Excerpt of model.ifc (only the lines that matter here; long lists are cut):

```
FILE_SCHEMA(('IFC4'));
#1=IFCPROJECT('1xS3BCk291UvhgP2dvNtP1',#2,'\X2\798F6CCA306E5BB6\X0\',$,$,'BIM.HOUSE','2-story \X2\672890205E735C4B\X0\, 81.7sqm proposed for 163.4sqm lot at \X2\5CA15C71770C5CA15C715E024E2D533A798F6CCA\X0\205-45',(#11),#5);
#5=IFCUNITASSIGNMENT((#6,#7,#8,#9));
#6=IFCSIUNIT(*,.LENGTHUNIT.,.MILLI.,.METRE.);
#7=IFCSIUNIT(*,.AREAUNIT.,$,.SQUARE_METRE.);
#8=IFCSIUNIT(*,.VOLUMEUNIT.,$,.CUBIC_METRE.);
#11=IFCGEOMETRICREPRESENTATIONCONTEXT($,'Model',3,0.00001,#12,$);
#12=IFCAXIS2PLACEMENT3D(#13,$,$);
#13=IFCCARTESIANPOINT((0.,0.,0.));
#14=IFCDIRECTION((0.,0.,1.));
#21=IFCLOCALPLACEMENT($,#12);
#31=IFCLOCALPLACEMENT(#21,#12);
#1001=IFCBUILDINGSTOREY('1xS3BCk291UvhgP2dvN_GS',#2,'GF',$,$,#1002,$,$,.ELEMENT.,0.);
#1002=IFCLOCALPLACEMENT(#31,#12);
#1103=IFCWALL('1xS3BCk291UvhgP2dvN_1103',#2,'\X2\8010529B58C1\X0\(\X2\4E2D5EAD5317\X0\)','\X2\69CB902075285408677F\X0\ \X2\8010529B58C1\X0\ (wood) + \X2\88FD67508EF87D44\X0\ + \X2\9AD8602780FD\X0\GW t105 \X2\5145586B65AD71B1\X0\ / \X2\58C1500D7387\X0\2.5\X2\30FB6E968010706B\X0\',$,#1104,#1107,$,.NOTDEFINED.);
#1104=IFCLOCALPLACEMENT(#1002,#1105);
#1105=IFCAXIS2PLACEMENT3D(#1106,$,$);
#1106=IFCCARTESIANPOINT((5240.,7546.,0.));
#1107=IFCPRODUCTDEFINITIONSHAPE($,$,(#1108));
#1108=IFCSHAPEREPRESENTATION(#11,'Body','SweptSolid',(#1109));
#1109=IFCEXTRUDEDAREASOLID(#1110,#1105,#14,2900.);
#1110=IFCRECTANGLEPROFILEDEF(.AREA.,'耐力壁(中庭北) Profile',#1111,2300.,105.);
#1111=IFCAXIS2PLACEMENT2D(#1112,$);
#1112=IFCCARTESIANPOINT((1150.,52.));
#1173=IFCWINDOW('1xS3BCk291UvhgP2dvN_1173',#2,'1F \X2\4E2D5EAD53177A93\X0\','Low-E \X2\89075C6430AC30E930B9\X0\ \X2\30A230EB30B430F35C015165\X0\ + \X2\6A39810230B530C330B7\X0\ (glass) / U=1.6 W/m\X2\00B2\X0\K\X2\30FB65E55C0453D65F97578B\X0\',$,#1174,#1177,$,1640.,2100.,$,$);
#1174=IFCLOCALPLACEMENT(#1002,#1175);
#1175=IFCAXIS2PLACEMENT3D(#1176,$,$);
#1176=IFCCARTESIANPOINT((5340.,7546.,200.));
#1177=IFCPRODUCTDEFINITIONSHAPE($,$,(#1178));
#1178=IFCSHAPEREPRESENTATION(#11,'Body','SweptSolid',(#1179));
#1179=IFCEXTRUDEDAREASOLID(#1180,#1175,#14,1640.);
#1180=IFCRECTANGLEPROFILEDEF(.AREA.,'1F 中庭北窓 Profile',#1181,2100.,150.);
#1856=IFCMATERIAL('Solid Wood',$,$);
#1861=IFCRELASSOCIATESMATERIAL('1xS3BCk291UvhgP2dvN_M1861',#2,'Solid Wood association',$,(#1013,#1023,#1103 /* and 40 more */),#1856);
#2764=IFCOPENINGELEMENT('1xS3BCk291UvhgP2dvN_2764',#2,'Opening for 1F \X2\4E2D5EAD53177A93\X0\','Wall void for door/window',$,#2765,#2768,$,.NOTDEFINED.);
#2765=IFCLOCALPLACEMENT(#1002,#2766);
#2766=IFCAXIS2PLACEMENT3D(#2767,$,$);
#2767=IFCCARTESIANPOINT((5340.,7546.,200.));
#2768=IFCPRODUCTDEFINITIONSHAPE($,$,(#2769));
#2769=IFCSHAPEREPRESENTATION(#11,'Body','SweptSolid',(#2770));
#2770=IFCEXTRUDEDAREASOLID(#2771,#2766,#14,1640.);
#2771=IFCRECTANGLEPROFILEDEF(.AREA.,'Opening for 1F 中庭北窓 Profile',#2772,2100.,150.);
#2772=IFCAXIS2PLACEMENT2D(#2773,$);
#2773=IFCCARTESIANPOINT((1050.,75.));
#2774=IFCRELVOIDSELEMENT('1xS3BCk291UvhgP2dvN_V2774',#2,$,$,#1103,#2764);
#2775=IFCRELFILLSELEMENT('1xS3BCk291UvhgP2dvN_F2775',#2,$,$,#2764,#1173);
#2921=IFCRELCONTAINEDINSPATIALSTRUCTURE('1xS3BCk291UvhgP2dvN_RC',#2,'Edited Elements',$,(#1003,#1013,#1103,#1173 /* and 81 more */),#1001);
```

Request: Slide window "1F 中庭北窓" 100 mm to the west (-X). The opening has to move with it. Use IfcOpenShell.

```python
import ifcopenshell
import ifcopenshell.api.geometry
import ifcopenshell.util.placement

model = ifcopenshell.open("model.ifc")

window = model.by_id(1173)
opening = window.FillsVoids[0].RelatingOpeningElement
wall = opening.VoidsElements[0].RelatingBuildingElement

wall_matrix = ifcopenshell.util.placement.get_local_placement(wall.ObjectPlacement)
shift = wall_matrix[:3, 0] * -100.0
before = ifcopenshell.util.placement.get_local_placement(window.ObjectPlacement)[:3, 3].copy()

# The window is not placed relative to its opening, so move both.
for product in (opening, window):
    matrix = ifcopenshell.util.placement.get_local_placement(product.ObjectPlacement)
    matrix[:3, 3] += shift
    ifcopenshell.api.geometry.edit_object_placement(model, product=product, matrix=matrix, is_si=False)

after = ifcopenshell.util.placement.get_local_placement(window.ObjectPlacement)[:3, 3]
print("window moved by", (after - before).round(3) + 0.0)

model.write("model-out.ifc")
```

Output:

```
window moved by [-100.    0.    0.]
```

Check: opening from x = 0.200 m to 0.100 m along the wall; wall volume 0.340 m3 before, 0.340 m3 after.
